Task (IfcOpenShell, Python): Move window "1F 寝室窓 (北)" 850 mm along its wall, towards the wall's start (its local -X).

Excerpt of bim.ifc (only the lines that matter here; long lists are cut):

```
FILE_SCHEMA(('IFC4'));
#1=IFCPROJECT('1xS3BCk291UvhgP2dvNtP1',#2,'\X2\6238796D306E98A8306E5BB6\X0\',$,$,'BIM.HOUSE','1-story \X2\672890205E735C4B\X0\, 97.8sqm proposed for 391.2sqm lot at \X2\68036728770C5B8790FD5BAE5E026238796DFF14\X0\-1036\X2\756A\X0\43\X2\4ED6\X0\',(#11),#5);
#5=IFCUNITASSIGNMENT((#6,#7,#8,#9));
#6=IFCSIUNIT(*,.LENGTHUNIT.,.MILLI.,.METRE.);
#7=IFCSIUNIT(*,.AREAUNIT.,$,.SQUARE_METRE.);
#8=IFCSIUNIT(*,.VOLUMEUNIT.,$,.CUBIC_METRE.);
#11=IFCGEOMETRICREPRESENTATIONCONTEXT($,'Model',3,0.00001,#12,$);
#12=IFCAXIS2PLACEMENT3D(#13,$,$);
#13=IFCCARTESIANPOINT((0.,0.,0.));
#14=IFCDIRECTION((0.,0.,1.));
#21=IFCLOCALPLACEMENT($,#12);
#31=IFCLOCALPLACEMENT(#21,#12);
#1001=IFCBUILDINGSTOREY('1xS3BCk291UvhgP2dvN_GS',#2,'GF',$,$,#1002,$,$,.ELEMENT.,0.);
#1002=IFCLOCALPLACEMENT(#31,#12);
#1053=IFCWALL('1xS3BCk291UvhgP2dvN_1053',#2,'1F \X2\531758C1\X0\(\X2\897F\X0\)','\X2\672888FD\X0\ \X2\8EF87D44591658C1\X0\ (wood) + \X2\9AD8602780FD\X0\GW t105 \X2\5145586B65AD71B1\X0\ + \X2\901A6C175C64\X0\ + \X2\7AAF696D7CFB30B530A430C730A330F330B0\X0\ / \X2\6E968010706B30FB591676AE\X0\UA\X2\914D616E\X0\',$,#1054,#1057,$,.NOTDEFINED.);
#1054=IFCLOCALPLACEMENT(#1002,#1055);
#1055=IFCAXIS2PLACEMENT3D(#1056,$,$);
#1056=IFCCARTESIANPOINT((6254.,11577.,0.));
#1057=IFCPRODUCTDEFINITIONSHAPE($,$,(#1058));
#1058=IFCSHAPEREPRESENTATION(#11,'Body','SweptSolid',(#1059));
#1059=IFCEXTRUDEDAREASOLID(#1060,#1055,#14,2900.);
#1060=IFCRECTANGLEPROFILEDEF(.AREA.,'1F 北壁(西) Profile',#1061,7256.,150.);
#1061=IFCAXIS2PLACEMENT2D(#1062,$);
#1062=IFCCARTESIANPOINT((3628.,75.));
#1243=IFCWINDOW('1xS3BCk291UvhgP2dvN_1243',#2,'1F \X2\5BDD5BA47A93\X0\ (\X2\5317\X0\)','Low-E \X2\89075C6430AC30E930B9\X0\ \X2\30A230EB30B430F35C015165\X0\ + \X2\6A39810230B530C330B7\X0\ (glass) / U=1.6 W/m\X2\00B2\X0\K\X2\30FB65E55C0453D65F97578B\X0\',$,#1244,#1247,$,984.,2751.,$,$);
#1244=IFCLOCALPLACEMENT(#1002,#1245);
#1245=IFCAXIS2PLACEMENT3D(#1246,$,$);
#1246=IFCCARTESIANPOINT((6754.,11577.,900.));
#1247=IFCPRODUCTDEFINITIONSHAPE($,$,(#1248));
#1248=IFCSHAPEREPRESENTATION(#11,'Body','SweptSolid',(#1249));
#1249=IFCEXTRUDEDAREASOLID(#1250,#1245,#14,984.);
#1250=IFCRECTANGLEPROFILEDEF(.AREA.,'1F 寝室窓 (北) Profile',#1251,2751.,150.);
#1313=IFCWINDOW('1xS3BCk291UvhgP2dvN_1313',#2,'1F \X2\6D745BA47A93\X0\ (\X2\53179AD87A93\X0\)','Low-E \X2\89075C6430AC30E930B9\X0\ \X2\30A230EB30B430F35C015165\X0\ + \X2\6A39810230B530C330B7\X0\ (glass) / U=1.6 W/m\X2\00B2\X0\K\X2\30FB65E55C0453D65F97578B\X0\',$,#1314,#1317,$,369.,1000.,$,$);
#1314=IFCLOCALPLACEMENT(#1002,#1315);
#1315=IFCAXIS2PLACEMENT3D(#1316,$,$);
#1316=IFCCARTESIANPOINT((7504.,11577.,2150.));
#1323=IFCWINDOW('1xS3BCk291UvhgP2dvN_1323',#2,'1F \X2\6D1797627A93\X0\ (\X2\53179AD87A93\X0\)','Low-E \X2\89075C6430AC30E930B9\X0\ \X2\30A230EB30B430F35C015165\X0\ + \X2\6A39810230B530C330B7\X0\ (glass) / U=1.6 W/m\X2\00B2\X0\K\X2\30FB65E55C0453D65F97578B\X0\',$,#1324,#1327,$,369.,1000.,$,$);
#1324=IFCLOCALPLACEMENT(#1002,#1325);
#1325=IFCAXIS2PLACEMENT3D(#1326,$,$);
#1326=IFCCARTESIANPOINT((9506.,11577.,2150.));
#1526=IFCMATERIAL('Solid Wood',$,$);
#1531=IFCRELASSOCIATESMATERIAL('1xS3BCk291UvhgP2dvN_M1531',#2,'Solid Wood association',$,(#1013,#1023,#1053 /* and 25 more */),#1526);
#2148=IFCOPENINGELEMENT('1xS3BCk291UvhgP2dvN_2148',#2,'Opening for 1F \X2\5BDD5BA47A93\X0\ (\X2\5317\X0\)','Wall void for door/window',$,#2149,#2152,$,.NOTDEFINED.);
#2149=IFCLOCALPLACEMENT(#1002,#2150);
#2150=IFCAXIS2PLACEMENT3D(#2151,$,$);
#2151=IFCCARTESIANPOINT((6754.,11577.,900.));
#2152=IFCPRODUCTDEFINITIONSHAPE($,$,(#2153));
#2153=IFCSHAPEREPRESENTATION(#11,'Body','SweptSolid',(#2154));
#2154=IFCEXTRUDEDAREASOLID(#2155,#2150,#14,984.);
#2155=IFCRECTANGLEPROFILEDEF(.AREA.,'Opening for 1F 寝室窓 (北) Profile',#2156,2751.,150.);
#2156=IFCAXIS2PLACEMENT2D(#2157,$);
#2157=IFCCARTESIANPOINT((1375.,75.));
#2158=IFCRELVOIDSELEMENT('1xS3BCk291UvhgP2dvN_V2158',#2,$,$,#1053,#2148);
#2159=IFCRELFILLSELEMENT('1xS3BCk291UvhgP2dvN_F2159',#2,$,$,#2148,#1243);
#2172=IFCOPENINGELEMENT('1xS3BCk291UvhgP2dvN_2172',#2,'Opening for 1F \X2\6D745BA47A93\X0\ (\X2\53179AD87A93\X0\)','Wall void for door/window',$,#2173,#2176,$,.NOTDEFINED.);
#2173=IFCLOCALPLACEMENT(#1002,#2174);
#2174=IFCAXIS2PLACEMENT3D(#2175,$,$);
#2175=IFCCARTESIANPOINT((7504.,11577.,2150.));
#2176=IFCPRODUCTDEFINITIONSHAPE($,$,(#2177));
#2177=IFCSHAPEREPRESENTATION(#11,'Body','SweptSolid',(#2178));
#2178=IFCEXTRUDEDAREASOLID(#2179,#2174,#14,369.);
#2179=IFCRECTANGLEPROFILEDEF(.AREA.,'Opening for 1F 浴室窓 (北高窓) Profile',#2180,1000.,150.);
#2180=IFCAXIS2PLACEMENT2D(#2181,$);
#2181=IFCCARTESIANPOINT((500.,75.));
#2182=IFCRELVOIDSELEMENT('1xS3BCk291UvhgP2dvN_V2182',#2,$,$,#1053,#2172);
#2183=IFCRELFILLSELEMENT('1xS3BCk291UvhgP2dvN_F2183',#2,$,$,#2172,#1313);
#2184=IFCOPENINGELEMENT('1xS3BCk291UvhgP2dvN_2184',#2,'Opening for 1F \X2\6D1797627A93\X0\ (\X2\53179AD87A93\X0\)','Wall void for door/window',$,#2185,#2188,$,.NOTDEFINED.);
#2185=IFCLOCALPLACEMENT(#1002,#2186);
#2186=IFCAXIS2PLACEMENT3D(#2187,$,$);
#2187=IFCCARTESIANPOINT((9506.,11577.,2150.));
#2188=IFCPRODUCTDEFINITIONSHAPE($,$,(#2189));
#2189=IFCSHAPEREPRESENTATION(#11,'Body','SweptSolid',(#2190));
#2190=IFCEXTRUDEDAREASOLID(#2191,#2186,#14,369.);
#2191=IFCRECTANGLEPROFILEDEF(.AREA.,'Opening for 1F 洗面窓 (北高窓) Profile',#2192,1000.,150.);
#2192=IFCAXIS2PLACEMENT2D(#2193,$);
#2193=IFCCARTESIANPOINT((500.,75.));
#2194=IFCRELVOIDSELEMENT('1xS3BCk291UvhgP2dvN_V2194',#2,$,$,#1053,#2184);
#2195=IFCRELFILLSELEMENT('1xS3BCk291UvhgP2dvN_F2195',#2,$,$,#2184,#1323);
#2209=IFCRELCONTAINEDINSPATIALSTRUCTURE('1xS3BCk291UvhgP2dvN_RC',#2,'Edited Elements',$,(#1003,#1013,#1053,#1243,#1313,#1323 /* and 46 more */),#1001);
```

```python
import ifcopenshell
import ifcopenshell.api.geometry
import ifcopenshell.util.placement

model = ifcopenshell.open("bim.ifc")

window = model.by_id(1243)
opening = window.FillsVoids[0].RelatingOpeningElement
wall = opening.VoidsElements[0].RelatingBuildingElement

wall_matrix = ifcopenshell.util.placement.get_local_placement(wall.ObjectPlacement)
shift = wall_matrix[:3, 0] * -850.0
before = ifcopenshell.util.placement.get_local_placement(window.ObjectPlacement)[:3, 3].copy()

# The window is not placed relative to its opening, so move both.
for product in (opening, window):
    matrix = ifcopenshell.util.placement.get_local_placement(product.ObjectPlacement)
    matrix[:3, 3] += shift
    ifcopenshell.api.geometry.edit_object_placement(model, product=product, matrix=matrix, is_si=False)

after = ifcopenshell.util.placement.get_local_placement(window.ObjectPlacement)[:3, 3]
print("window moved by", (after - before).round(3) + 0.0)

model.write("bim_v2.ifc")
```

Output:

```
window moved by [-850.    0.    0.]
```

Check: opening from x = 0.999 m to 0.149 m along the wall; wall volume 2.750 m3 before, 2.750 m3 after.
